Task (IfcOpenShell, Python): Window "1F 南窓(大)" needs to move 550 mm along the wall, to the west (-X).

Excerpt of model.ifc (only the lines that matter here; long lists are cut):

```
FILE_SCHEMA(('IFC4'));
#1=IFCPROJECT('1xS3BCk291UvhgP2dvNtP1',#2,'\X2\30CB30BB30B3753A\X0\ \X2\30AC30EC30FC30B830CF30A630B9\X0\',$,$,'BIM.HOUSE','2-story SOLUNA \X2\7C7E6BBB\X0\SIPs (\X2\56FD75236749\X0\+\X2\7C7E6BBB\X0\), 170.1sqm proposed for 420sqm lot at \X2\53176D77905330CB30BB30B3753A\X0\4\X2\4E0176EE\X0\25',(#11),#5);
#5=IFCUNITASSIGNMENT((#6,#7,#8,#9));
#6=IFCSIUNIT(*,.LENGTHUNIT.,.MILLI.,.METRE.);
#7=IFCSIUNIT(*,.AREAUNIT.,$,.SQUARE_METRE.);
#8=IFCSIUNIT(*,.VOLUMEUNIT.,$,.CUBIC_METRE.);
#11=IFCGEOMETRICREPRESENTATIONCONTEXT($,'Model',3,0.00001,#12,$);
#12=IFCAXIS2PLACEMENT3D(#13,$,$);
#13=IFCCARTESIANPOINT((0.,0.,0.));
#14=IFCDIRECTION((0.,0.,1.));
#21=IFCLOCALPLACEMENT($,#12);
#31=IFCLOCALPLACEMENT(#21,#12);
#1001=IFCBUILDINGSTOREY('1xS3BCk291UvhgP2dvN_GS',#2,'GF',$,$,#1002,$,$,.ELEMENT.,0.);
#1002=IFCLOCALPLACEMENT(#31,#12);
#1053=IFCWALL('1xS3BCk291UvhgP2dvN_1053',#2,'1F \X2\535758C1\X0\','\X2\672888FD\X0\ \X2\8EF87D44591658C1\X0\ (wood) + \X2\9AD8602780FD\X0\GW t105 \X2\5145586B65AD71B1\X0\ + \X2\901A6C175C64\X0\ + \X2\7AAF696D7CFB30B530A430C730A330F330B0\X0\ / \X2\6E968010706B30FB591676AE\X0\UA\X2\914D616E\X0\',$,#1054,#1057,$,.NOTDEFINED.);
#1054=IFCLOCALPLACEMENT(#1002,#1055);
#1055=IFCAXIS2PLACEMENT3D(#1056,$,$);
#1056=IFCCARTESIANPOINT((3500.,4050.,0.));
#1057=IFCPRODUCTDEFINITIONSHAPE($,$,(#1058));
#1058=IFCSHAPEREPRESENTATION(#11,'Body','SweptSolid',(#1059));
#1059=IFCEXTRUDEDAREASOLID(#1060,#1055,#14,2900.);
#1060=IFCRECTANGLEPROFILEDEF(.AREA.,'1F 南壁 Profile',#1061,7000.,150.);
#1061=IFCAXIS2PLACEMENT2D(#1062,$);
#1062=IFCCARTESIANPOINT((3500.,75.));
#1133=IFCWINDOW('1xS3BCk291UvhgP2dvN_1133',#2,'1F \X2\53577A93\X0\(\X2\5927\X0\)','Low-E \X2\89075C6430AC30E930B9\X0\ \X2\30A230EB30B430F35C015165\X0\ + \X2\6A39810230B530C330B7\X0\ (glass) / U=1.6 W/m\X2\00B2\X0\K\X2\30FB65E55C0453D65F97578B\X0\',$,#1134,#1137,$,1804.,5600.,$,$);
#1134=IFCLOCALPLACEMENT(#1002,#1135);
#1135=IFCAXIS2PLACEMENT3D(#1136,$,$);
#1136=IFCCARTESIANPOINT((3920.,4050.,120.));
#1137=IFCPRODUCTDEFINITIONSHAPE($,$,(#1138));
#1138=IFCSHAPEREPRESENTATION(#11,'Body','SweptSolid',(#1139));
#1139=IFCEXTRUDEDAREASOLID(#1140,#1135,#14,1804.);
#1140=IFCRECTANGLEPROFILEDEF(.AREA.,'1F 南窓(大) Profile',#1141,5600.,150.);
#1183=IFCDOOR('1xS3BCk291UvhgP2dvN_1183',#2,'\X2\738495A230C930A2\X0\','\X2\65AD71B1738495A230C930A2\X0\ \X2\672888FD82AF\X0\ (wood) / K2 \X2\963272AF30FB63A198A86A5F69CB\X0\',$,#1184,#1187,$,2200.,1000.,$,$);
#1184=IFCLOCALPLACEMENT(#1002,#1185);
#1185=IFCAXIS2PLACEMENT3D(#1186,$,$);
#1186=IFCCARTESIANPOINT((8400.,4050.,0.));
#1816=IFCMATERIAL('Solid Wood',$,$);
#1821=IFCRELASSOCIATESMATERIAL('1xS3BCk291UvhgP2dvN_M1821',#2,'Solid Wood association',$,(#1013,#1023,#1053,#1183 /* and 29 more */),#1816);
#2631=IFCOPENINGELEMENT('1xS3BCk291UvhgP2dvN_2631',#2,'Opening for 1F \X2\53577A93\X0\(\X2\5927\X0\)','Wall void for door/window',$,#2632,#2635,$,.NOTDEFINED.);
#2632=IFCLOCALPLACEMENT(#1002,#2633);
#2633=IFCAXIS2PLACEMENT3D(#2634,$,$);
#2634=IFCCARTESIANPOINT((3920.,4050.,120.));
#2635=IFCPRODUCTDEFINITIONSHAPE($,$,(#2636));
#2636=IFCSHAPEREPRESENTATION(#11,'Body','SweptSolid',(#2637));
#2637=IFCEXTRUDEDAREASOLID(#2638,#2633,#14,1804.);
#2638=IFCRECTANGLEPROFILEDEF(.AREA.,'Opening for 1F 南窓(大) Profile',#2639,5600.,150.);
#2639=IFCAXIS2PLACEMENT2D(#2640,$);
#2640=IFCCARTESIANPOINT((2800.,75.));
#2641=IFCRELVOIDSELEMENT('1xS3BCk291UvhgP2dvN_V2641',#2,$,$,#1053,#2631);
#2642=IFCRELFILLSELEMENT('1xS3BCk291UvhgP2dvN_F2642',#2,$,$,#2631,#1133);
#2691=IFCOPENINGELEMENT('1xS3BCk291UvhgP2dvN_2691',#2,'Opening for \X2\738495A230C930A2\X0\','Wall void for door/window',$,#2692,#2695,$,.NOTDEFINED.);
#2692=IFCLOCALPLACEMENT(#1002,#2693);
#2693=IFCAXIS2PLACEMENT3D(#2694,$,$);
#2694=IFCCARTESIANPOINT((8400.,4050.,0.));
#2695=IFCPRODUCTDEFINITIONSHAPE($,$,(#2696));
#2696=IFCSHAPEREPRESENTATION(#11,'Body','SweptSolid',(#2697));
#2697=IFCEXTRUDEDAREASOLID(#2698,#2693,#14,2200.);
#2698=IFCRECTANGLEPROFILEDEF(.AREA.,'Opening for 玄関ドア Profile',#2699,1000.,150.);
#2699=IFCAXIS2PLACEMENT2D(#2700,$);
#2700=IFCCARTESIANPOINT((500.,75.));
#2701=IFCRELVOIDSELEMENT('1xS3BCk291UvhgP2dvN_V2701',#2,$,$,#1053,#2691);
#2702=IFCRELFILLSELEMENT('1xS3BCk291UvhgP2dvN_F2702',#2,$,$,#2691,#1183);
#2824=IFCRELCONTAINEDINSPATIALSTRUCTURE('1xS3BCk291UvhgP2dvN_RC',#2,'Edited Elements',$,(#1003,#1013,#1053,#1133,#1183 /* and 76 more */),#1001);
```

```python
import ifcopenshell
import ifcopenshell.api.geometry
import ifcopenshell.util.placement
import ifcopenshell.util.unit

model = ifcopenshell.open("model.ifc")
unit_scale = ifcopenshell.util.unit.calculate_unit_scale(model)

window = model.by_guid("1xS3BCk291UvhgP2dvN_1133")
opening = window.FillsVoids[0].RelatingOpeningElement
wall = opening.VoidsElements[0].RelatingBuildingElement

wall_matrix = ifcopenshell.util.placement.get_local_placement(wall.ObjectPlacement)
shift = wall_matrix[:3, 0] * -0.55 / unit_scale
before = ifcopenshell.util.placement.get_local_placement(window.ObjectPlacement)[:3, 3].copy()

# The window is not placed relative to its opening, so move both.
for product in (opening, window):
    matrix = ifcopenshell.util.placement.get_local_placement(product.ObjectPlacement)
    matrix[:3, 3] += shift
    ifcopenshell.api.geometry.edit_object_placement(model, product=product, matrix=matrix, is_si=False)

after = ifcopenshell.util.placement.get_local_placement(window.ObjectPlacement)[:3, 3]
print("window moved by", (after - before).round(3) + 0.0)

model.write("model_edited.ifc")
```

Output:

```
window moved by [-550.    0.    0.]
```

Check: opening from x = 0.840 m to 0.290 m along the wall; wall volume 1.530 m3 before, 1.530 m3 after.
